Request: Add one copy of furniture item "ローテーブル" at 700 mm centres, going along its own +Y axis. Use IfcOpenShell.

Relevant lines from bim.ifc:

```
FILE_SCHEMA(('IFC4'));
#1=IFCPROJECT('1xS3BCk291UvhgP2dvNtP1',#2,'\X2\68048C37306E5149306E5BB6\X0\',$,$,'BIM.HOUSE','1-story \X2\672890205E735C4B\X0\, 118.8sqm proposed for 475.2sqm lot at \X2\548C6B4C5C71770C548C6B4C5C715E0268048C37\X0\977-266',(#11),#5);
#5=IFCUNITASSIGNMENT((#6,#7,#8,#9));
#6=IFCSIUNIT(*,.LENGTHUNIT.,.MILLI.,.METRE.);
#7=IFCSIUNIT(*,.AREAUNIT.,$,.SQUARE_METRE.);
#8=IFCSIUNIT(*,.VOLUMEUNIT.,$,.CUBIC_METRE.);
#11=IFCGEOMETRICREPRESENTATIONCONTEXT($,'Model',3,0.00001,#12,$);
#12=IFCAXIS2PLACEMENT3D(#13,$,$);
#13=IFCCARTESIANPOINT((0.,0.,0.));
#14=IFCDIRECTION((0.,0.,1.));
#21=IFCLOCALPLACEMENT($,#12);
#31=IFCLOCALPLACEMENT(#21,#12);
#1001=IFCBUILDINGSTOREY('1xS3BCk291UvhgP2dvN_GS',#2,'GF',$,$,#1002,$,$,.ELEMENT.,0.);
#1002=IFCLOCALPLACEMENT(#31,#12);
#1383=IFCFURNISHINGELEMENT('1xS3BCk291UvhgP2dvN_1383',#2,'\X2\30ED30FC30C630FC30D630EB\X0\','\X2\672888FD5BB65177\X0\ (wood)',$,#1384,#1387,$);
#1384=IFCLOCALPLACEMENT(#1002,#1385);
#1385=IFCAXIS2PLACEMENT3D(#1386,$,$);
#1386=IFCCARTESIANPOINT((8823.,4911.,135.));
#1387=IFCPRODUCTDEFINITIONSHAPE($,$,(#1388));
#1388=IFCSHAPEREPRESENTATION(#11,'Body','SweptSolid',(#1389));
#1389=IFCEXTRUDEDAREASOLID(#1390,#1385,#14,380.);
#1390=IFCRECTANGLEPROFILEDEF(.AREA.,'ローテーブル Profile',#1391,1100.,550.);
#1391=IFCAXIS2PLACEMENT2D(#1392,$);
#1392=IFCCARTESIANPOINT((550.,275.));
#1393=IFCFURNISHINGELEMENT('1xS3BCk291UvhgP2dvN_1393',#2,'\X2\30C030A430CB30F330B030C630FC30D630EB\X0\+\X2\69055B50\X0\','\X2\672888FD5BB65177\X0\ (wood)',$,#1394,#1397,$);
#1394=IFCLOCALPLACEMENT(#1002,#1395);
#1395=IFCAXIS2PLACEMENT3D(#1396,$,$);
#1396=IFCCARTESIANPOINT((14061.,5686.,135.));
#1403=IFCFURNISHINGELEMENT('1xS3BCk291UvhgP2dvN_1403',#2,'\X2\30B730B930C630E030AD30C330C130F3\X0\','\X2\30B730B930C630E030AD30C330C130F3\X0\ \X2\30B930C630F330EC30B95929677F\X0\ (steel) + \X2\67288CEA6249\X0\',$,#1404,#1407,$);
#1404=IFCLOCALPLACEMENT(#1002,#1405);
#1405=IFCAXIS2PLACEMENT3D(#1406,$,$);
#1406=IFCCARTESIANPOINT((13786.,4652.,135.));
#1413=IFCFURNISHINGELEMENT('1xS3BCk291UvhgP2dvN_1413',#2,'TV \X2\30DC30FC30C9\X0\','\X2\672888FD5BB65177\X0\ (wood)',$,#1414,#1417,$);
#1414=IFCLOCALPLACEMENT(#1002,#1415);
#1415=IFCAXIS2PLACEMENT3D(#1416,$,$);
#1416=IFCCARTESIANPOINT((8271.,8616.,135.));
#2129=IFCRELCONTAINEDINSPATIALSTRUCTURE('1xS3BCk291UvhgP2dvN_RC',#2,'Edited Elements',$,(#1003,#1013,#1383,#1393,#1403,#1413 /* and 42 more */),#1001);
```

```python
import ifcopenshell
import ifcopenshell.api.geometry
import ifcopenshell.api.root
import ifcopenshell.util.element
import ifcopenshell.util.placement

model = ifcopenshell.open("bim.ifc")


def reuse_history(source, copy):
    """copy_class also copies each property set's owner history, people and application; keep the originals."""
    for rel in copy.IsDefinedBy:
        if rel.is_a("IfcRelDefinesByProperties") and (history := rel.RelatingPropertyDefinition.OwnerHistory):
            rel.RelatingPropertyDefinition.OwnerHistory = source.OwnerHistory
            ifcopenshell.util.element.remove_deep2(model, history)


source = model.by_guid("1xS3BCk291UvhgP2dvN_1383")
base = ifcopenshell.util.placement.get_local_placement(source.ObjectPlacement)
step = base[:3, 1] * 700.0

for i in range(1, 2):
    copy = ifcopenshell.api.root.copy_class(model, product=source)
    copy.Representation = ifcopenshell.util.element.copy_deep(
        model, source.Representation, exclude=["IfcGeometricRepresentationContext", "IfcRepresentationMap"]
    )
    reuse_history(source, copy)
    matrix = base.copy()
    matrix[:3, 3] += i * step
    print("added at", matrix[:3, 3].round(3) + 0.0)
    ifcopenshell.api.geometry.edit_object_placement(model, product=copy, matrix=matrix, is_si=False)

model.write("bim_updated.ifc")
```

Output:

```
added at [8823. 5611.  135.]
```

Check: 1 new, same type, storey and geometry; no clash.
